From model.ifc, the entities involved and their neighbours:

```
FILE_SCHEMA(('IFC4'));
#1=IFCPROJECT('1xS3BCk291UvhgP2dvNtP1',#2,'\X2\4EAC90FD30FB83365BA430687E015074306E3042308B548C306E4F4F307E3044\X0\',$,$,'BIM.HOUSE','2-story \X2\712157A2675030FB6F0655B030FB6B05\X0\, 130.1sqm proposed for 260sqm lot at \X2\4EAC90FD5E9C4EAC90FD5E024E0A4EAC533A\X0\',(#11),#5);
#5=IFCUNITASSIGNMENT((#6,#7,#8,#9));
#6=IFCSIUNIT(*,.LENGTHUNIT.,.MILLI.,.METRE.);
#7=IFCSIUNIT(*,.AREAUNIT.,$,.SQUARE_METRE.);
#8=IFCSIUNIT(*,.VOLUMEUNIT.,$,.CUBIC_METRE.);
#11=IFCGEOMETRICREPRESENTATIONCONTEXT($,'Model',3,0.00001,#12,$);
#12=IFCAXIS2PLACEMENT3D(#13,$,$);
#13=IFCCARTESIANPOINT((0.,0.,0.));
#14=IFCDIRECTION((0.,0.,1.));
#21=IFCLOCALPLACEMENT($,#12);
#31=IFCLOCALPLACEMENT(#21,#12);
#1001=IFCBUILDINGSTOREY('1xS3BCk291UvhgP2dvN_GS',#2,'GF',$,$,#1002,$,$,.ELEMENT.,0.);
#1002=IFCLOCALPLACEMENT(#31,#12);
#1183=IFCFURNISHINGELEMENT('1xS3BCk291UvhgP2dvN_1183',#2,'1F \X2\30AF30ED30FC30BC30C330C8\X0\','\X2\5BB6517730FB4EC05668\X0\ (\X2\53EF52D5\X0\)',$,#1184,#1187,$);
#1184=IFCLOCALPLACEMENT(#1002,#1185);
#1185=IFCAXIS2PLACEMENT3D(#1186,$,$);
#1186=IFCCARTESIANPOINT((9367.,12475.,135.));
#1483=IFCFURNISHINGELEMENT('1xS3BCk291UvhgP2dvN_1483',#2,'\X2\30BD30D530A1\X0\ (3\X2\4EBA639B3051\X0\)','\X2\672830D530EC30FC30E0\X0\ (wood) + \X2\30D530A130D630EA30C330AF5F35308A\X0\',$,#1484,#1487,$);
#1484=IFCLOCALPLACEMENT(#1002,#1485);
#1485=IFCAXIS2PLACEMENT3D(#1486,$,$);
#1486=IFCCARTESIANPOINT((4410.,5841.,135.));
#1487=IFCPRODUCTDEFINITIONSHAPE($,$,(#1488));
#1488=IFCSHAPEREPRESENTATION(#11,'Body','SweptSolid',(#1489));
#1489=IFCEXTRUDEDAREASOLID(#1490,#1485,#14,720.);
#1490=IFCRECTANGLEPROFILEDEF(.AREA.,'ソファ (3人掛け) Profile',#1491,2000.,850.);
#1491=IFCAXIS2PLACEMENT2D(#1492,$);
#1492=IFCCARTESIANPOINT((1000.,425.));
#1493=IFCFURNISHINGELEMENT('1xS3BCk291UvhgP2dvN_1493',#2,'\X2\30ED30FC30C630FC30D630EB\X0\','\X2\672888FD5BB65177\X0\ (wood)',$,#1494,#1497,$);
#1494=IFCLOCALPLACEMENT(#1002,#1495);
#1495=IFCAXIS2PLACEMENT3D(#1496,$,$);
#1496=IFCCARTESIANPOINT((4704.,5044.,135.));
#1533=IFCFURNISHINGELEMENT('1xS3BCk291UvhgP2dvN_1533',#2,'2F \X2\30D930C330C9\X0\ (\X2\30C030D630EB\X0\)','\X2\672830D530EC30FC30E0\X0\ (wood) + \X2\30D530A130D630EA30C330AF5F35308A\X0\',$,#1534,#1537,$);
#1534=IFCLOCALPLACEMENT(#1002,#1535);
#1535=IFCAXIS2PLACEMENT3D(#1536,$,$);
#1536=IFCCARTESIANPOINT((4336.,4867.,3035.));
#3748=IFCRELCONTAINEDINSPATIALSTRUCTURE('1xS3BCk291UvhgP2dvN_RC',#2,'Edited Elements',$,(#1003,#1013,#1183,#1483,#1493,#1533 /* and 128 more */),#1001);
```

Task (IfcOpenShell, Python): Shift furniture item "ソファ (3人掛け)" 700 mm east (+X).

```python
import ifcopenshell
import ifcopenshell.api.geometry
import ifcopenshell.util.placement
import ifcopenshell.util.unit

model = ifcopenshell.open("model.ifc")
unit_scale = ifcopenshell.util.unit.calculate_unit_scale(model)

item = model.by_id(1483)
matrix = ifcopenshell.util.placement.get_local_placement(item.ObjectPlacement)
matrix[0, 3] += 0.7 / unit_scale
ifcopenshell.api.geometry.edit_object_placement(model, product=item, matrix=matrix, is_si=False)

print(ifcopenshell.util.placement.get_local_placement(item.ObjectPlacement).round(3) + 0.0)

model.write("model_rev.ifc")
```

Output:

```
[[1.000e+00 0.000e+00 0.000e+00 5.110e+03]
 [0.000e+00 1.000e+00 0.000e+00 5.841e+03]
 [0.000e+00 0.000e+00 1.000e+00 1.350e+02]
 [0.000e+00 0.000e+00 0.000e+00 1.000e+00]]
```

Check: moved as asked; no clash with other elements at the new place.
